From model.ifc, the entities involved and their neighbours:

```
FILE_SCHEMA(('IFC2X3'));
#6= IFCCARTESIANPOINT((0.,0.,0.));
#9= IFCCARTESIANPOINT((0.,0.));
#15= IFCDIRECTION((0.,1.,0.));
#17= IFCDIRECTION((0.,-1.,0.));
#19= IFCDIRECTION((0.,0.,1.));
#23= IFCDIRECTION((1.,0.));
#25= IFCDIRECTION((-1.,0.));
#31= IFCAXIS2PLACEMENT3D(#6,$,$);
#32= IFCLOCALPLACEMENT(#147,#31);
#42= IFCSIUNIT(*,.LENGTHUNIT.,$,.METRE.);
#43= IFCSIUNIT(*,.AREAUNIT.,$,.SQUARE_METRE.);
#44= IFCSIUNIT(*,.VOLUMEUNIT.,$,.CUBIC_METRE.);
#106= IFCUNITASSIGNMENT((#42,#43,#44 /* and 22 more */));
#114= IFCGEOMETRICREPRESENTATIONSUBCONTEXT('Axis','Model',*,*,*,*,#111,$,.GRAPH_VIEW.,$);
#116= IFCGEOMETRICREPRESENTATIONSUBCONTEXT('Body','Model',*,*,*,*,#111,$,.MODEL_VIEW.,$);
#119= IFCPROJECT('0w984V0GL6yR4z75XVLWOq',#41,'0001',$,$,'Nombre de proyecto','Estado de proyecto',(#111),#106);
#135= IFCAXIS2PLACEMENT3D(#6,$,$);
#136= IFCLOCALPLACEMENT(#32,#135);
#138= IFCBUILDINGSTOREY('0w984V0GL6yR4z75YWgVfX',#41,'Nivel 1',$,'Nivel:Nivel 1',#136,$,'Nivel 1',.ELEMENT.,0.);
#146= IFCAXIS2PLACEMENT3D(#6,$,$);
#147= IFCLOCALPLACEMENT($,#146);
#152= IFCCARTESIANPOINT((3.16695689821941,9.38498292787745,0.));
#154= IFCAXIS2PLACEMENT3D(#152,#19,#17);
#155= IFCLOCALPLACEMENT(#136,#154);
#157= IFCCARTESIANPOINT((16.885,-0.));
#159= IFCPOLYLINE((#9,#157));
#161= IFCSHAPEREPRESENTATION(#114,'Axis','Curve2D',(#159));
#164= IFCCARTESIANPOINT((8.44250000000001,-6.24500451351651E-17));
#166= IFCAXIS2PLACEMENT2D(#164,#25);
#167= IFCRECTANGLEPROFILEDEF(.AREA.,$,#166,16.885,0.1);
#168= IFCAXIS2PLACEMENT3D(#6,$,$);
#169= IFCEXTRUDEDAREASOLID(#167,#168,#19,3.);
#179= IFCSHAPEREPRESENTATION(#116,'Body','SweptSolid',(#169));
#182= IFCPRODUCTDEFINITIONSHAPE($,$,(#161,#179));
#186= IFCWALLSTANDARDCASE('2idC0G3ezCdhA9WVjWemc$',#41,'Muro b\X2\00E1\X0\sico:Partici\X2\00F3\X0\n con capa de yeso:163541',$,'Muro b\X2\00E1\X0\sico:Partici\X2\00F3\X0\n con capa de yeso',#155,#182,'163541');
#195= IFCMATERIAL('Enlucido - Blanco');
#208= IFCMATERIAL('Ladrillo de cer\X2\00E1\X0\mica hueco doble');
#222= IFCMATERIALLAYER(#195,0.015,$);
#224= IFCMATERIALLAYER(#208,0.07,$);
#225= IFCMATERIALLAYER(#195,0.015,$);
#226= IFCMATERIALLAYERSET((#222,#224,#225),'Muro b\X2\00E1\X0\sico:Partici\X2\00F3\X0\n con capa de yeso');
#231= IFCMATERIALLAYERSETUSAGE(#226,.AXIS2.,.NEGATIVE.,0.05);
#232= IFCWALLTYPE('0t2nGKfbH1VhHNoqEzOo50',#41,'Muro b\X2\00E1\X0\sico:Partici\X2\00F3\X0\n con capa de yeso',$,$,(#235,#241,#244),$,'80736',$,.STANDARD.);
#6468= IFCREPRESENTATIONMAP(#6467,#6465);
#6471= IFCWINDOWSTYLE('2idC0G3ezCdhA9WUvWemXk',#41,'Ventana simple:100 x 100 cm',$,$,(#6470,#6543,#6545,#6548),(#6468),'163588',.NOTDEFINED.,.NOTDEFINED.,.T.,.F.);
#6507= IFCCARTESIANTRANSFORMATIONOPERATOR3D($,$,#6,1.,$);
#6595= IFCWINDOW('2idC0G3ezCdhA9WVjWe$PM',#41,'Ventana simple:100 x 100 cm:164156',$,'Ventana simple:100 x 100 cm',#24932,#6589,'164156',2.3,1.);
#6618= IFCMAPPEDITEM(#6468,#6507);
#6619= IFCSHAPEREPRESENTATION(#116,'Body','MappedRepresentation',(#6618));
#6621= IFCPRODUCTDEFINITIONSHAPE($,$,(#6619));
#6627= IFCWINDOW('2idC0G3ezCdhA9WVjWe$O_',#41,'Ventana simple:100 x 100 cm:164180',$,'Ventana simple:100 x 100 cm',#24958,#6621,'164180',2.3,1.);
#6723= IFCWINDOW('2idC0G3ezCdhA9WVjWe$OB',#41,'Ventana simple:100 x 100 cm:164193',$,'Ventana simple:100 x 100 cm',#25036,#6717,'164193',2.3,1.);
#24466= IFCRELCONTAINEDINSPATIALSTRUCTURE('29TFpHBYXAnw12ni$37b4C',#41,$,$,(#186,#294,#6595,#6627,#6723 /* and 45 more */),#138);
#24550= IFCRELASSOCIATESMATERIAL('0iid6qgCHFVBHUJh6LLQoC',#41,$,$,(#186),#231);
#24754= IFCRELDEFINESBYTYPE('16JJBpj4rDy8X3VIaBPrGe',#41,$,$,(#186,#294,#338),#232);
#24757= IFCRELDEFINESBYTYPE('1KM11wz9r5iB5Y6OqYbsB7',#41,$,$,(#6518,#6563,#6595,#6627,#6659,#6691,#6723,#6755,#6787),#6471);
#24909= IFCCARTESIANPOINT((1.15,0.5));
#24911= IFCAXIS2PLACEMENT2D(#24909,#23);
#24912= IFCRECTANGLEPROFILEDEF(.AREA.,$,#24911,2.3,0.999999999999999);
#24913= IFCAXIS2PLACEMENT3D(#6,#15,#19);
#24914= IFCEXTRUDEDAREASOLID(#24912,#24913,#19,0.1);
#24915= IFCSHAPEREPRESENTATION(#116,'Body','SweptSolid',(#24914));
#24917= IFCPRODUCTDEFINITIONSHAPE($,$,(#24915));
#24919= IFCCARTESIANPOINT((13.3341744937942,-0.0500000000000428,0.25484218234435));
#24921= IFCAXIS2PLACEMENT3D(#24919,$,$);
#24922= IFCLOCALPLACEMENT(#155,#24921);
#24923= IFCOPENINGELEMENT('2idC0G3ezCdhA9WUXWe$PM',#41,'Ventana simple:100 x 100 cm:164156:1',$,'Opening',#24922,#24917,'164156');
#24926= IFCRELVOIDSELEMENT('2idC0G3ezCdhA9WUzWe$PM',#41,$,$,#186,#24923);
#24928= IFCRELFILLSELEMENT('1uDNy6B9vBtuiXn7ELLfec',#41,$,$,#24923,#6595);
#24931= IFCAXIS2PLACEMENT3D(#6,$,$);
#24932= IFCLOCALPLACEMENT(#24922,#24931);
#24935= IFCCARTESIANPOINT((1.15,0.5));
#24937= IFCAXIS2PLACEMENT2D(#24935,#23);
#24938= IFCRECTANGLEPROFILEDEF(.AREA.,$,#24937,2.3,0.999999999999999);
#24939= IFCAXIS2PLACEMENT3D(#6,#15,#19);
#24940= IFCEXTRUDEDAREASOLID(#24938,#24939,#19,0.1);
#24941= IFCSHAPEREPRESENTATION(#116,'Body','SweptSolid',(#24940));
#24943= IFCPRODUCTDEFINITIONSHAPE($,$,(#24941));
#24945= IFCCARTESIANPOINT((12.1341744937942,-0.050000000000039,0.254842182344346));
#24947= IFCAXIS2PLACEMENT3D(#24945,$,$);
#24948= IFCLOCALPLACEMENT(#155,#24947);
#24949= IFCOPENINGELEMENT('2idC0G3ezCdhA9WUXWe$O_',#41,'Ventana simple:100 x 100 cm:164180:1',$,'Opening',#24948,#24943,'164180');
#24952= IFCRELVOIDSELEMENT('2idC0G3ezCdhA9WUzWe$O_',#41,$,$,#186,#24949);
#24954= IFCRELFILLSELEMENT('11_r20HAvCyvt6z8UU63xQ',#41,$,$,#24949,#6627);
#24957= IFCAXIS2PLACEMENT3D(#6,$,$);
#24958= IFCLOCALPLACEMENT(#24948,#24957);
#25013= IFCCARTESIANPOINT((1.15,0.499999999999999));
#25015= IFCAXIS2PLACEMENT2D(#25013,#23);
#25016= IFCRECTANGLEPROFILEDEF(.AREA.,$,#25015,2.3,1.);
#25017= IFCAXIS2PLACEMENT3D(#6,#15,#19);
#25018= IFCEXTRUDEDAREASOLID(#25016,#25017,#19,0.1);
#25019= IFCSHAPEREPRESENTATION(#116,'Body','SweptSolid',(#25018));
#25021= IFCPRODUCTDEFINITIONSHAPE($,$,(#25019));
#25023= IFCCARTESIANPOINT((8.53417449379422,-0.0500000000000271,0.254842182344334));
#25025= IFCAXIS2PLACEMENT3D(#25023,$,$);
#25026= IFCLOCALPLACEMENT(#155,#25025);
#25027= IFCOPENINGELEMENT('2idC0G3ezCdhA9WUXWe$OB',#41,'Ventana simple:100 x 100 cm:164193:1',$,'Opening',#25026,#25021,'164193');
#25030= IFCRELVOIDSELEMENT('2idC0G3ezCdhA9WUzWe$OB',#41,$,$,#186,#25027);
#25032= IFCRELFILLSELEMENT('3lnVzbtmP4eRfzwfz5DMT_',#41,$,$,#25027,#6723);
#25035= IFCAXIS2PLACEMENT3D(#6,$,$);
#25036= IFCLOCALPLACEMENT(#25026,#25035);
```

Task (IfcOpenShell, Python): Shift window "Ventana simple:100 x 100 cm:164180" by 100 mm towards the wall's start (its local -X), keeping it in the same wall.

```python
import ifcopenshell
import ifcopenshell.api.geometry
import ifcopenshell.util.placement
import ifcopenshell.util.unit

model = ifcopenshell.open("model.ifc")
unit_scale = ifcopenshell.util.unit.calculate_unit_scale(model)

window = model.by_guid("2idC0G3ezCdhA9WVjWe$O_")
opening = window.FillsVoids[0].RelatingOpeningElement
wall = opening.VoidsElements[0].RelatingBuildingElement

wall_matrix = ifcopenshell.util.placement.get_local_placement(wall.ObjectPlacement)
shift = wall_matrix[:3, 0] * -0.1 / unit_scale
before = ifcopenshell.util.placement.get_local_placement(window.ObjectPlacement)[:3, 3].copy()

# The window is placed relative to its opening, so it follows when the opening moves.
matrix = ifcopenshell.util.placement.get_local_placement(opening.ObjectPlacement)
matrix[:3, 3] += shift
ifcopenshell.api.geometry.edit_object_placement(
    model, product=opening, matrix=matrix, is_si=False, should_transform_children=True
)

after = ifcopenshell.util.placement.get_local_placement(window.ObjectPlacement)[:3, 3]
print("window moved by", (after - before).round(3) + 0.0)

model.write("model_rev.ifc")
```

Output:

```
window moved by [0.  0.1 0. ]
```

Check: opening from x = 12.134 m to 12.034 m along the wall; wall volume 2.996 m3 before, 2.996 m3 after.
